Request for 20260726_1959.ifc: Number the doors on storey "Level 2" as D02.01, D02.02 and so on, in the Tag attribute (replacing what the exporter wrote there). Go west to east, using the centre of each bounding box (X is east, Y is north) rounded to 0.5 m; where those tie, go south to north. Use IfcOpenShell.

First a look at what the model holds.

```python
import ifcopenshell
import ifcopenshell.util.element
import ifcopenshell.util.placement

model = ifcopenshell.open("20260726_1959.ifc")
print(model.schema)
storey = next(s for s in model.by_type("IfcBuildingStorey") if s.Name == "Level 2")
doors = [e for e in ifcopenshell.util.element.get_decomposition(storey) if e.is_a("IfcDoor")]
for e in sorted(doors, key=lambda e: e.id()):
    origin = ifcopenshell.util.placement.get_local_placement(e.ObjectPlacement)[:3, 3]
    print(e.id(), e.Tag, e.Name, origin.round(2) + 0.0, sep=" | ")
```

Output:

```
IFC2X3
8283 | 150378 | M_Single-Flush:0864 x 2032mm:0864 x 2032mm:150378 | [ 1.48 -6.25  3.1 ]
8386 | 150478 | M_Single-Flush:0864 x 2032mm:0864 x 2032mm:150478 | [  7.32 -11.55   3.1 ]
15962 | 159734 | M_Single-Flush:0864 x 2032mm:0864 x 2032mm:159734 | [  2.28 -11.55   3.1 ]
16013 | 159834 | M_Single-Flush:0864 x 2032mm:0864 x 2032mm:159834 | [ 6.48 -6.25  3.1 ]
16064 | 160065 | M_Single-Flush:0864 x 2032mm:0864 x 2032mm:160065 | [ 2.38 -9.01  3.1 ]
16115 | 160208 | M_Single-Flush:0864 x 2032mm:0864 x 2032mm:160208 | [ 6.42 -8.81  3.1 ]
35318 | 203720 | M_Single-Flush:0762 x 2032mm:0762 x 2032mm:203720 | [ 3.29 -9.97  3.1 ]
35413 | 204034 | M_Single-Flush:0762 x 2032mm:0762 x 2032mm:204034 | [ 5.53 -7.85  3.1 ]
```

```python
import ifcopenshell
import ifcopenshell.geom
import ifcopenshell.util.element
import ifcopenshell.util.shape

model = ifcopenshell.open("20260726_1959.ifc")
settings = ifcopenshell.geom.settings()
settings.set("use-world-coords", True)


def centre(element):
    shape = ifcopenshell.geom.create_shape(settings, element)
    return ifcopenshell.util.shape.get_bbox_centroid(shape.geometry)


storey = next(s for s in model.by_type("IfcBuildingStorey") if s.Name == "Level 2")
doors = [e for e in ifcopenshell.util.element.get_decomposition(storey) if e.is_a("IfcDoor")]

# Insertion points can sit at a corner or the storey origin, so sort by the geometry (in metres).
centres = {e: centre(e) for e in doors}
doors.sort(key=lambda e: (round(centres[e][0] / 0.5), centres[e][1]))

for i, e in enumerate(doors, start=1):
    number = f"D02.{i:02d}"
    e.Tag = number
    print(e.id(), number)

model.write("20260726_1959_rev.ifc")
```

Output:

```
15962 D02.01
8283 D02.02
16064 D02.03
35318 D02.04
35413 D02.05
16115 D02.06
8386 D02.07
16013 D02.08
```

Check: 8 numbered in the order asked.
